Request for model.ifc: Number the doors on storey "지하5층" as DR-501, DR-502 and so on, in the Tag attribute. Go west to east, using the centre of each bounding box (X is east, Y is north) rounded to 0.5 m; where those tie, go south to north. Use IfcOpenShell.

First a look at what the model holds.

```python
import ifcopenshell
import ifcopenshell.util.element
import ifcopenshell.util.placement

model = ifcopenshell.open("model.ifc")
print(model.schema)
storey = next(s for s in model.by_type("IfcBuildingStorey") if s.Name == "지하5층")
doors = [e for e in ifcopenshell.util.element.get_decomposition(storey) if e.is_a("IfcDoor")]
for e in sorted(doors, key=lambda e: e.id()):
    origin = ifcopenshell.util.placement.get_local_placement(e.ObjectPlacement)[:3, 3]
    print(e.id(), e.Tag, e.Name, origin.round(2) + 0.0, sep=" | ")
```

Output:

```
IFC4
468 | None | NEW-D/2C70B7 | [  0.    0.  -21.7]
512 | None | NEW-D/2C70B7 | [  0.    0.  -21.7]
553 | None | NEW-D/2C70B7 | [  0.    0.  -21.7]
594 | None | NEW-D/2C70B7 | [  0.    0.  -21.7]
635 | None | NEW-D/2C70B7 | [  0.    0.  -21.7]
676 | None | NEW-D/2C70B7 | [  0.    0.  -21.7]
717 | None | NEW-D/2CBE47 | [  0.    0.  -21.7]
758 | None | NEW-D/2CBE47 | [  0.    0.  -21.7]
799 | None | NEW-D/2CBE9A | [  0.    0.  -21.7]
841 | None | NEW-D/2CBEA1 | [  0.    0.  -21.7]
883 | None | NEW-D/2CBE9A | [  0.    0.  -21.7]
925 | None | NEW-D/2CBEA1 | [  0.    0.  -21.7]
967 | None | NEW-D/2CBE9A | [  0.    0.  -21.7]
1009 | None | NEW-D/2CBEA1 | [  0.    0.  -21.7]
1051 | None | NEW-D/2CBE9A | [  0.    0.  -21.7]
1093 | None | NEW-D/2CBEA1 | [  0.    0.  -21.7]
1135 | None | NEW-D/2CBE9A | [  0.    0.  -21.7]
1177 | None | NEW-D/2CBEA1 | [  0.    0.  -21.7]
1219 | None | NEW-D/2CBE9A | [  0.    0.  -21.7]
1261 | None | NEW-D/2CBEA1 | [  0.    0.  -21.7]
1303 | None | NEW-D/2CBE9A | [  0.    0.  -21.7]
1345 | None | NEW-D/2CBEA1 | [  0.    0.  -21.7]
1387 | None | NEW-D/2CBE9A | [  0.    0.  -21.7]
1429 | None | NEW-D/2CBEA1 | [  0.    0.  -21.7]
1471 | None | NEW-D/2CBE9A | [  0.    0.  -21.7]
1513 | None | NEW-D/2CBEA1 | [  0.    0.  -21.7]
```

```python
import ifcopenshell
import ifcopenshell.geom
import ifcopenshell.util.element
import ifcopenshell.util.shape

model = ifcopenshell.open("model.ifc")
settings = ifcopenshell.geom.settings()
settings.set("use-world-coords", True)


def centre(element):
    shape = ifcopenshell.geom.create_shape(settings, element)
    return ifcopenshell.util.shape.get_bbox_centroid(shape.geometry)


storey = next(s for s in model.by_type("IfcBuildingStorey") if s.Name == "지하5층")
doors = [e for e in ifcopenshell.util.element.get_decomposition(storey) if e.is_a("IfcDoor")]

# Insertion points can sit at a corner or the storey origin, so sort by the geometry (in metres).
centres = {e: centre(e) for e in doors}
doors.sort(key=lambda e: (round(centres[e][0] / 0.5), centres[e][1]))

for i, e in enumerate(doors, start=1):
    number = f"DR-5{i:02d}"
    e.Tag = number
    print(e.id(), number)

model.write("model_v2.ifc")
```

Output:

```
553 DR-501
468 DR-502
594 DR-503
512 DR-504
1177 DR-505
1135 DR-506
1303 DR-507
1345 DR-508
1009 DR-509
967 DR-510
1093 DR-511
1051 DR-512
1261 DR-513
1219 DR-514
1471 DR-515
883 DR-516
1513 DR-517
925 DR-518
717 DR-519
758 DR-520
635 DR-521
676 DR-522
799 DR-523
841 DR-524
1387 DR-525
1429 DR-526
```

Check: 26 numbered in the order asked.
